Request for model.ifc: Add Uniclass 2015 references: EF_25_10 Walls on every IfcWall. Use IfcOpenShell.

First a look at what the model holds.

```python
import ifcopenshell

model = ifcopenshell.open("model.ifc")
print(model.schema)
print("classifications:", [c.Name for c in model.by_type("IfcClassification")])
for ifc_class in ("IfcDoor", "IfcRoof", "IfcStair", "IfcWall", "IfcWindow"):
    print(ifc_class, len(model.by_type(ifc_class)))
```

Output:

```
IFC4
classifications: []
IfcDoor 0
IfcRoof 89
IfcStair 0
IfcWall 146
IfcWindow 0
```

```python
import ifcopenshell
import ifcopenshell.api.classification

model = ifcopenshell.open("model.ifc")

system = ifcopenshell.api.classification.add_classification(model, classification="Uniclass 2015")

codes = {
    "IfcWall": ("EF_25_10", "Walls"),
}
for ifc_class, (code, name) in codes.items():
    products = model.by_type(ifc_class)
    ifcopenshell.api.classification.add_reference(
        model, products=products, classification=system, identification=code, name=name
    )
    print(code, len(products))

model.write("model_rev.ifc")
```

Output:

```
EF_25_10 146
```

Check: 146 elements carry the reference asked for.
